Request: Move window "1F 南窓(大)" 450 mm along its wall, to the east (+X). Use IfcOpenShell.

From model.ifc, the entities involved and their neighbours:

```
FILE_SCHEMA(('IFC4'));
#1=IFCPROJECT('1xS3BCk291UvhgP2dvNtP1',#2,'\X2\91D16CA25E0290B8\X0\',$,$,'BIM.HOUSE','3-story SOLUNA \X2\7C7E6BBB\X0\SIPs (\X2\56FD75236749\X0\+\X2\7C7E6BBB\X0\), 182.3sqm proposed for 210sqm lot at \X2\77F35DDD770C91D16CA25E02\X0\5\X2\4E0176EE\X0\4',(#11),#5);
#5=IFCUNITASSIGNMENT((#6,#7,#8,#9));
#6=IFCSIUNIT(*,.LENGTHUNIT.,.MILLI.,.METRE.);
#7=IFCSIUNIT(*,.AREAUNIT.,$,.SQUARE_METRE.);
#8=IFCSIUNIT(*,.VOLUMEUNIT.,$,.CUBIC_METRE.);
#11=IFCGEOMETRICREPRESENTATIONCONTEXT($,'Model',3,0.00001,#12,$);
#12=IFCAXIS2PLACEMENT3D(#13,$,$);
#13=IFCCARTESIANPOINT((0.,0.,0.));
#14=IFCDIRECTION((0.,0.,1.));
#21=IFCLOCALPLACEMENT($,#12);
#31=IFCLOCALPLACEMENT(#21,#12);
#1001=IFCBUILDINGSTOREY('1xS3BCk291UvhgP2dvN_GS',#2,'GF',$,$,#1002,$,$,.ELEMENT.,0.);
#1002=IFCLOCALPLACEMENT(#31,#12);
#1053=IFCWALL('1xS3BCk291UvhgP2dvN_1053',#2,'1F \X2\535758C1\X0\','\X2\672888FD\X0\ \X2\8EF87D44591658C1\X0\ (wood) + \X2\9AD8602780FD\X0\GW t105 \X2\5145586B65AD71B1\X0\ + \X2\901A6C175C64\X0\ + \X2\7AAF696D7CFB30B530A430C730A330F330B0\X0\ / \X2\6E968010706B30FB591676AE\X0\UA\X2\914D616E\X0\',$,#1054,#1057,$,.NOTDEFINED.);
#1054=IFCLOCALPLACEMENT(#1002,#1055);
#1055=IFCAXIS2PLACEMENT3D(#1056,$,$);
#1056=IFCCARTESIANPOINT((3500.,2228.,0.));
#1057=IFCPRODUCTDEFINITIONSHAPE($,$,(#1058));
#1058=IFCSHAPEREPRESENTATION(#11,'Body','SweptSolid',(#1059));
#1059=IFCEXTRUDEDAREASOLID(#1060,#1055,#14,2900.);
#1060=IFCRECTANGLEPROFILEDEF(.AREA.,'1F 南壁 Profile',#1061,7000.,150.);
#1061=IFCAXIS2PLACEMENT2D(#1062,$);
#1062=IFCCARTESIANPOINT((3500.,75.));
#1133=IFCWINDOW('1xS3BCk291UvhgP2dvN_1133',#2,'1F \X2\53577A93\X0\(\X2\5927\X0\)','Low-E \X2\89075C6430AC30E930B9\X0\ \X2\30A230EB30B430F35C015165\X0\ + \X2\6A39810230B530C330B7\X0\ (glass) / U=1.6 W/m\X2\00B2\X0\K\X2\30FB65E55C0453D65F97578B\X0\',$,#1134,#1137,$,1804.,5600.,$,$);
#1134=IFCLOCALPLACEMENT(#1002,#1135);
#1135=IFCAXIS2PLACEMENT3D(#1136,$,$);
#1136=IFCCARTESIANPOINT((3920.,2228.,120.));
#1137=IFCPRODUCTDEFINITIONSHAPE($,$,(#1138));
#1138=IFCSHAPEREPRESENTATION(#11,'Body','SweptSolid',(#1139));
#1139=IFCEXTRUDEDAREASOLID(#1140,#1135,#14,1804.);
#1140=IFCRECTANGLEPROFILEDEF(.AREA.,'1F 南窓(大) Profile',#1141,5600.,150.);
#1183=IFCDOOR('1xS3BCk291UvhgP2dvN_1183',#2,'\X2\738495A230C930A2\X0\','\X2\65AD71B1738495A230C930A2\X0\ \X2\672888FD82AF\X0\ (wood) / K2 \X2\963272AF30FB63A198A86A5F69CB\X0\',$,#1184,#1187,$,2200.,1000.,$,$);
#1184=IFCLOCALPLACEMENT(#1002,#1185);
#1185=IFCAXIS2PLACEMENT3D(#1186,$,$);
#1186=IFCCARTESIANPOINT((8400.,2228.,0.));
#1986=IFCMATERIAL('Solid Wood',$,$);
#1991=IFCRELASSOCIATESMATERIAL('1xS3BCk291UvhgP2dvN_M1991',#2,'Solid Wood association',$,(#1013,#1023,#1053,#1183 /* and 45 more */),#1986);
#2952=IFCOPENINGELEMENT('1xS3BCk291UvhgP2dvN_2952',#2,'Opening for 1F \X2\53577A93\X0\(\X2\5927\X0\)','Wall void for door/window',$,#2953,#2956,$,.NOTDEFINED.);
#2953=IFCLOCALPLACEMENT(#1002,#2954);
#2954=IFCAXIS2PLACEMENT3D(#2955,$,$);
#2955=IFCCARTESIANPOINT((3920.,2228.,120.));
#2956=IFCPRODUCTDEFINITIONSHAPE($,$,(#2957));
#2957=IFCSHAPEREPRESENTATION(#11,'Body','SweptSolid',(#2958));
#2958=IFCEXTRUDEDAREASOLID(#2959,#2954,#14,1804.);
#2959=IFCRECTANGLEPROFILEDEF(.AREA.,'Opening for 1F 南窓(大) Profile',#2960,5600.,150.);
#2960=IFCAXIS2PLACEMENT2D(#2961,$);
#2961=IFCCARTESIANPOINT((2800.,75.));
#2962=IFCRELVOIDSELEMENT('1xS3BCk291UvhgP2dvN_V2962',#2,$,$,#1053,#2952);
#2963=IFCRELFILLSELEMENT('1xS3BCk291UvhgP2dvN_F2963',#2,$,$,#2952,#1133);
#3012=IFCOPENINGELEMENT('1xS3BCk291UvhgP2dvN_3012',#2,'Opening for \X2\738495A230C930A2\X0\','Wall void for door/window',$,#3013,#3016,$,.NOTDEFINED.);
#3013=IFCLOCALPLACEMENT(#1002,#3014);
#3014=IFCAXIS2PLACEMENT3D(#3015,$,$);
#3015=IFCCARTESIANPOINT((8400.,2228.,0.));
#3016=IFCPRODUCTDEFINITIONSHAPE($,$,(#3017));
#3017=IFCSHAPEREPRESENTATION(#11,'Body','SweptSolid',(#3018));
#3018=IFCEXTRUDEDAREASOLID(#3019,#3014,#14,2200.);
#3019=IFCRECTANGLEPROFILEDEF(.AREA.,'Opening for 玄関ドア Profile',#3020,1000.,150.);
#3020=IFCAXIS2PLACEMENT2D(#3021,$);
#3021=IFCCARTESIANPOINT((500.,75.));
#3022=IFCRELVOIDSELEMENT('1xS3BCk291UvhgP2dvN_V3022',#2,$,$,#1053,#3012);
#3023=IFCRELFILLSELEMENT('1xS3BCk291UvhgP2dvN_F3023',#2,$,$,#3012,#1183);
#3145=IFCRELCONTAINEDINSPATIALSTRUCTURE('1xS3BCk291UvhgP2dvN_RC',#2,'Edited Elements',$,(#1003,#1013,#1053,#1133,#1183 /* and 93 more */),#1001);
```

```python
import ifcopenshell
import ifcopenshell.api.geometry
import ifcopenshell.util.placement
import ifcopenshell.util.unit

model = ifcopenshell.open("model.ifc")
unit_scale = ifcopenshell.util.unit.calculate_unit_scale(model)

window = model.by_guid("1xS3BCk291UvhgP2dvN_1133")
opening = window.FillsVoids[0].RelatingOpeningElement
wall = opening.VoidsElements[0].RelatingBuildingElement

wall_matrix = ifcopenshell.util.placement.get_local_placement(wall.ObjectPlacement)
shift = wall_matrix[:3, 0] * 0.45 / unit_scale
before = ifcopenshell.util.placement.get_local_placement(window.ObjectPlacement)[:3, 3].copy()

# The window is not placed relative to its opening, so move both.
for product in (opening, window):
    matrix = ifcopenshell.util.placement.get_local_placement(product.ObjectPlacement)
    matrix[:3, 3] += shift
    ifcopenshell.api.geometry.edit_object_placement(model, product=product, matrix=matrix, is_si=False)

after = ifcopenshell.util.placement.get_local_placement(window.ObjectPlacement)[:3, 3]
print("window moved by", (after - before).round(3) + 0.0)

model.write("model_edited.ifc")
```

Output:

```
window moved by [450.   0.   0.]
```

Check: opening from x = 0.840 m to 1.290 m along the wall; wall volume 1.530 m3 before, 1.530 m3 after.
